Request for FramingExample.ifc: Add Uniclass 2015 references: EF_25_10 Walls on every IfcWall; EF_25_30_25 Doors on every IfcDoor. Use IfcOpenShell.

First a look at what the model holds.

```python
import ifcopenshell

model = ifcopenshell.open("FramingExample.ifc")
print(model.schema)
print("classifications:", [c.Name for c in model.by_type("IfcClassification")])
for ifc_class in ("IfcDoor", "IfcRoof", "IfcStair", "IfcWall", "IfcWindow"):
    print(ifc_class, len(model.by_type(ifc_class)))
```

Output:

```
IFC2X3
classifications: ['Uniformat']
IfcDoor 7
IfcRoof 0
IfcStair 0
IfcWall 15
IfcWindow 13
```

```python
import ifcopenshell
import ifcopenshell.api.classification

model = ifcopenshell.open("FramingExample.ifc")

# IFC2X3 requires Source and Edition and has no link from the project to the system.
system = model.create_entity("IfcClassification", Source="NBS", Edition="2015", Name="Uniclass 2015")

codes = {
    "IfcWall": ("EF_25_10", "Walls"),
    "IfcDoor": ("EF_25_30_25", "Doors"),
}
for ifc_class, (code, name) in codes.items():
    products = model.by_type(ifc_class)
    ifcopenshell.api.classification.add_reference(
        model, products=products, classification=system, identification=code, name=name
    )
    print(code, len(products))

model.write("FramingExample-out.ifc")
```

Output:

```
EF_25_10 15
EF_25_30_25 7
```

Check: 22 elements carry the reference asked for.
